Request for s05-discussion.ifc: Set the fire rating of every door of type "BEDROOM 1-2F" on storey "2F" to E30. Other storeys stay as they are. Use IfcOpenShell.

First a look at what the model holds.

```python
import ifcopenshell
import ifcopenshell.util.element

model = ifcopenshell.open("s05-discussion.ifc")
print(model.schema)
storey = next(s for s in model.by_type("IfcBuildingStorey") if s.Name == "2F")
doors = [e for e in ifcopenshell.util.element.get_decomposition(storey) if e.is_a("IfcDoor")]
seen = {}
for e in doors:
    element_type = ifcopenshell.util.element.get_type(e)
    key = (element_type.Name if element_type != e and element_type else None, ifcopenshell.util.element.get_pset(e, "Pset_DoorCommon", "FireRating"))
    seen[key] = seen.get(key, 0) + 1
for (name, value), count in sorted(seen.items(), key=str):
    print(count, "x", name, "|", value)
```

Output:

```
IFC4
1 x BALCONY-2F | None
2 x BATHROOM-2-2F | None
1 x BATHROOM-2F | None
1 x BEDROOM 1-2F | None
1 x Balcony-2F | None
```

```python
import ifcopenshell
import ifcopenshell.api.pset
import ifcopenshell.util.element

model = ifcopenshell.open("s05-discussion.ifc")

storey = next(s for s in model.by_type("IfcBuildingStorey") if s.Name == "2F")
doors = [e for e in ifcopenshell.util.element.get_decomposition(storey) if e.is_a("IfcDoor")]

count = 0
for e in doors:
    element_type = ifcopenshell.util.element.get_type(e)
    if element_type in (None, e) or element_type.Name != "BEDROOM 1-2F":
        continue
    # add_pset returns the element's existing set when there is one.
    pset = ifcopenshell.api.pset.add_pset(model, product=e, name="Pset_DoorCommon")
    ifcopenshell.api.pset.edit_pset(model, pset=pset, properties={"FireRating": "E30"})
    count += 1

print(count, "doors updated")

model.write("s05-discussion_v2.ifc")
```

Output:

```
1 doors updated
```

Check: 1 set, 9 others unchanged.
